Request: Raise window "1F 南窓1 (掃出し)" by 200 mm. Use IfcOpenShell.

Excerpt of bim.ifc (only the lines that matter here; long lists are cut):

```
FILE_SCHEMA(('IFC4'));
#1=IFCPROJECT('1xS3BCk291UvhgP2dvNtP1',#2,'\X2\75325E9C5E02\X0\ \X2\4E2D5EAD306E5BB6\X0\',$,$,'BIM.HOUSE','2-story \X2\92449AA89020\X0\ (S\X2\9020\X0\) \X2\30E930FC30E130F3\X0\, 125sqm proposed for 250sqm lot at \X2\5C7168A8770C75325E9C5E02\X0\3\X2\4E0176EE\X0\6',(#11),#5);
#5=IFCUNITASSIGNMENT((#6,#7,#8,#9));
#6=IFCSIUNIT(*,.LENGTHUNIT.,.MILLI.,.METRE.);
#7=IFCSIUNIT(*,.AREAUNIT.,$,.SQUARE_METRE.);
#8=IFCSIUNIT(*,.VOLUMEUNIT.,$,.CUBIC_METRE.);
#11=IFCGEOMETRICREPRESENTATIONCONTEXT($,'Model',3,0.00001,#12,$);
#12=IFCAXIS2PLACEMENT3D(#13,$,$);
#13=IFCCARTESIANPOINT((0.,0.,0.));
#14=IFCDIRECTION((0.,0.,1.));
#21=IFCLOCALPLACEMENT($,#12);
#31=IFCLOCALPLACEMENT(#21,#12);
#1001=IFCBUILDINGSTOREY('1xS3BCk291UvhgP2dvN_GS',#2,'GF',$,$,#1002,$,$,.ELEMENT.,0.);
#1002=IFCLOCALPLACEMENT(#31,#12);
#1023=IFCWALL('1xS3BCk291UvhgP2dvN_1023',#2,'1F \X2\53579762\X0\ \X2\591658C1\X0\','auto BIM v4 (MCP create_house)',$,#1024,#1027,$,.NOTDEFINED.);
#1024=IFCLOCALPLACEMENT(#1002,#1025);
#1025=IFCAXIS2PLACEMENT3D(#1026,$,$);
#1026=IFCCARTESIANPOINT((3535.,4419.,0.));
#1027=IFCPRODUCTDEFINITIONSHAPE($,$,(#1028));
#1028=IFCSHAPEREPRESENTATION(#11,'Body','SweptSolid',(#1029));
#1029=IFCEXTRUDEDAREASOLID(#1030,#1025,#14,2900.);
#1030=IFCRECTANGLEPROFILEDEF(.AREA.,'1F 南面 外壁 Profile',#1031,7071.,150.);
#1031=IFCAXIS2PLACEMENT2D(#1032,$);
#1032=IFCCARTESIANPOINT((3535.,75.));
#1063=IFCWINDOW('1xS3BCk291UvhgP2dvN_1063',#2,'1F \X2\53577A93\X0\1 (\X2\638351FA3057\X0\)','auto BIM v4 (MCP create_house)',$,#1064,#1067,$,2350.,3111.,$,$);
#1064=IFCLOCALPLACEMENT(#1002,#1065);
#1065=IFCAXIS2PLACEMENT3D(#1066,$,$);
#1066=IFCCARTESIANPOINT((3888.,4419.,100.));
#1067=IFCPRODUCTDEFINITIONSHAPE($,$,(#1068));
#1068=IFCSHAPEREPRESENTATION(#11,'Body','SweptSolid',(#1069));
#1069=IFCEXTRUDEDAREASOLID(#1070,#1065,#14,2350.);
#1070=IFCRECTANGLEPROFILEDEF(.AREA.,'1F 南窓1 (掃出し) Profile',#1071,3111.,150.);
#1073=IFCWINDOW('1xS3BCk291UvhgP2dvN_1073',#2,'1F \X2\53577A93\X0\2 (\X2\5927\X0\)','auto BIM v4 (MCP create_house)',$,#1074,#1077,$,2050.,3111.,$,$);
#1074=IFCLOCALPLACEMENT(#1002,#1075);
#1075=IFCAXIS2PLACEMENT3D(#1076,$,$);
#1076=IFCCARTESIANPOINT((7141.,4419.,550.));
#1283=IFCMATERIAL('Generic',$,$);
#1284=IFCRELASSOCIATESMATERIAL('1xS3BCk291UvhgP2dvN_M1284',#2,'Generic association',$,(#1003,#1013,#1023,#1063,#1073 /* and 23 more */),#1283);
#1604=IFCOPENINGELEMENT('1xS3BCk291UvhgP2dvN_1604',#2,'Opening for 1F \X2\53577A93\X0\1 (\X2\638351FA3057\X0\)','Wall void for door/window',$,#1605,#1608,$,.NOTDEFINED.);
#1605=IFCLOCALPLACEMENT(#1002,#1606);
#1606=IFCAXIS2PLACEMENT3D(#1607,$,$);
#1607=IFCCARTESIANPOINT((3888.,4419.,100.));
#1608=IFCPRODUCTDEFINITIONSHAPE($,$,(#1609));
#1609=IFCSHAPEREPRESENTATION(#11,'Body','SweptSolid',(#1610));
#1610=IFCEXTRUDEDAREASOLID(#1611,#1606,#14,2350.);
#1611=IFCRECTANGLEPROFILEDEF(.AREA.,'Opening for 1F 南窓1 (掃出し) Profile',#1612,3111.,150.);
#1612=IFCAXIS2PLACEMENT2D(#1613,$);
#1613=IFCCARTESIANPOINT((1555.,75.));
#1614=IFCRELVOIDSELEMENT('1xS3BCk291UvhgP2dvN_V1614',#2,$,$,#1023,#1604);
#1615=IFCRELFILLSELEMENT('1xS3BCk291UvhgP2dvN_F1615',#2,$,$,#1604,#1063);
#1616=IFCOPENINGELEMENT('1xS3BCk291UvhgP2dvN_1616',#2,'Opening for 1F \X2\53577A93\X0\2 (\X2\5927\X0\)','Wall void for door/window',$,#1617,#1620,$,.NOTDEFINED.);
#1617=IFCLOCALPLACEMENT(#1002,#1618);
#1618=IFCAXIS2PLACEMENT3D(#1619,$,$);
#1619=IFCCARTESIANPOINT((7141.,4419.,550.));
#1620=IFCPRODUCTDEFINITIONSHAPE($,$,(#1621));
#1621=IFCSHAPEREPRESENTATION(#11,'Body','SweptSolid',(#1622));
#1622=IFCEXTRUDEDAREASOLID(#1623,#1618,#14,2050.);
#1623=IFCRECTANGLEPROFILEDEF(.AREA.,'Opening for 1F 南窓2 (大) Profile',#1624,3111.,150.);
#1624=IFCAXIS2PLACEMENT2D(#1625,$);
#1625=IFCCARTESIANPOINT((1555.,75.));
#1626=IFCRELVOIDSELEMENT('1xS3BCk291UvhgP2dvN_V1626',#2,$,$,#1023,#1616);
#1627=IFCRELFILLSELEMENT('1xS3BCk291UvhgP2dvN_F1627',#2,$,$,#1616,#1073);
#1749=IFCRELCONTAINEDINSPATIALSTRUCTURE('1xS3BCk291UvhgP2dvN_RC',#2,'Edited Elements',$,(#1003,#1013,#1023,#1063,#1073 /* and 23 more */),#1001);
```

```python
import numpy as np
import ifcopenshell
import ifcopenshell.api.geometry
import ifcopenshell.util.placement
import ifcopenshell.util.unit

model = ifcopenshell.open("bim.ifc")
unit_scale = ifcopenshell.util.unit.calculate_unit_scale(model)

window = model.by_guid("1xS3BCk291UvhgP2dvN_1063")
opening = window.FillsVoids[0].RelatingOpeningElement
dz = 0.2 / unit_scale

shift = np.array([0.0, 0.0, dz])
# The window is not placed relative to its opening, so move both.
for product in (opening, window):
    matrix = ifcopenshell.util.placement.get_local_placement(product.ObjectPlacement)
    matrix[:3, 3] += shift
    ifcopenshell.api.geometry.edit_object_placement(model, product=product, matrix=matrix, is_si=False)

print(f"moved by {dz * unit_scale:+.3f} m")

model.write("bim_v2.ifc")
```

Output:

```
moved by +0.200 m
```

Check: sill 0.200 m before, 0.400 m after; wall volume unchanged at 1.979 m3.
